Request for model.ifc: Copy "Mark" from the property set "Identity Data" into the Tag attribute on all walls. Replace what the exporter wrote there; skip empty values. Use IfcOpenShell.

First a look at what the model holds.

```python
import ifcopenshell
import ifcopenshell.util.element

model = ifcopenshell.open("model.ifc")
print(model.schema)
walls = model.by_type("IfcWall")
print(len(walls), "walls")
for e in walls[:8]:
    source = ifcopenshell.util.element.get_pset(e, "Identity Data", "Mark")
    target = e.Tag
    print(e.id(), repr(source), repr(target), sep=" | ")
```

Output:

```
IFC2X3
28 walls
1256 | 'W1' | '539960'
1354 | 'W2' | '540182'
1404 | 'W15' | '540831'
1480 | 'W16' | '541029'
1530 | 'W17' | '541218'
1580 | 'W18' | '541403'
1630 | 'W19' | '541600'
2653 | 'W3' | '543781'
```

```python
import ifcopenshell
import ifcopenshell.util.element

model = ifcopenshell.open("model.ifc")

count = 0
for e in model.by_type("IfcWall"):
    value = ifcopenshell.util.element.get_pset(e, "Identity Data", "Mark")
    current = e.Tag
    if not value or not value.strip() or current == value:
        continue
    e.Tag = value
    count += 1

print(count, "walls updated")

model.write("model_v2.ifc")
```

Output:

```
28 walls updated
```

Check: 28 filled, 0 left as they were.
